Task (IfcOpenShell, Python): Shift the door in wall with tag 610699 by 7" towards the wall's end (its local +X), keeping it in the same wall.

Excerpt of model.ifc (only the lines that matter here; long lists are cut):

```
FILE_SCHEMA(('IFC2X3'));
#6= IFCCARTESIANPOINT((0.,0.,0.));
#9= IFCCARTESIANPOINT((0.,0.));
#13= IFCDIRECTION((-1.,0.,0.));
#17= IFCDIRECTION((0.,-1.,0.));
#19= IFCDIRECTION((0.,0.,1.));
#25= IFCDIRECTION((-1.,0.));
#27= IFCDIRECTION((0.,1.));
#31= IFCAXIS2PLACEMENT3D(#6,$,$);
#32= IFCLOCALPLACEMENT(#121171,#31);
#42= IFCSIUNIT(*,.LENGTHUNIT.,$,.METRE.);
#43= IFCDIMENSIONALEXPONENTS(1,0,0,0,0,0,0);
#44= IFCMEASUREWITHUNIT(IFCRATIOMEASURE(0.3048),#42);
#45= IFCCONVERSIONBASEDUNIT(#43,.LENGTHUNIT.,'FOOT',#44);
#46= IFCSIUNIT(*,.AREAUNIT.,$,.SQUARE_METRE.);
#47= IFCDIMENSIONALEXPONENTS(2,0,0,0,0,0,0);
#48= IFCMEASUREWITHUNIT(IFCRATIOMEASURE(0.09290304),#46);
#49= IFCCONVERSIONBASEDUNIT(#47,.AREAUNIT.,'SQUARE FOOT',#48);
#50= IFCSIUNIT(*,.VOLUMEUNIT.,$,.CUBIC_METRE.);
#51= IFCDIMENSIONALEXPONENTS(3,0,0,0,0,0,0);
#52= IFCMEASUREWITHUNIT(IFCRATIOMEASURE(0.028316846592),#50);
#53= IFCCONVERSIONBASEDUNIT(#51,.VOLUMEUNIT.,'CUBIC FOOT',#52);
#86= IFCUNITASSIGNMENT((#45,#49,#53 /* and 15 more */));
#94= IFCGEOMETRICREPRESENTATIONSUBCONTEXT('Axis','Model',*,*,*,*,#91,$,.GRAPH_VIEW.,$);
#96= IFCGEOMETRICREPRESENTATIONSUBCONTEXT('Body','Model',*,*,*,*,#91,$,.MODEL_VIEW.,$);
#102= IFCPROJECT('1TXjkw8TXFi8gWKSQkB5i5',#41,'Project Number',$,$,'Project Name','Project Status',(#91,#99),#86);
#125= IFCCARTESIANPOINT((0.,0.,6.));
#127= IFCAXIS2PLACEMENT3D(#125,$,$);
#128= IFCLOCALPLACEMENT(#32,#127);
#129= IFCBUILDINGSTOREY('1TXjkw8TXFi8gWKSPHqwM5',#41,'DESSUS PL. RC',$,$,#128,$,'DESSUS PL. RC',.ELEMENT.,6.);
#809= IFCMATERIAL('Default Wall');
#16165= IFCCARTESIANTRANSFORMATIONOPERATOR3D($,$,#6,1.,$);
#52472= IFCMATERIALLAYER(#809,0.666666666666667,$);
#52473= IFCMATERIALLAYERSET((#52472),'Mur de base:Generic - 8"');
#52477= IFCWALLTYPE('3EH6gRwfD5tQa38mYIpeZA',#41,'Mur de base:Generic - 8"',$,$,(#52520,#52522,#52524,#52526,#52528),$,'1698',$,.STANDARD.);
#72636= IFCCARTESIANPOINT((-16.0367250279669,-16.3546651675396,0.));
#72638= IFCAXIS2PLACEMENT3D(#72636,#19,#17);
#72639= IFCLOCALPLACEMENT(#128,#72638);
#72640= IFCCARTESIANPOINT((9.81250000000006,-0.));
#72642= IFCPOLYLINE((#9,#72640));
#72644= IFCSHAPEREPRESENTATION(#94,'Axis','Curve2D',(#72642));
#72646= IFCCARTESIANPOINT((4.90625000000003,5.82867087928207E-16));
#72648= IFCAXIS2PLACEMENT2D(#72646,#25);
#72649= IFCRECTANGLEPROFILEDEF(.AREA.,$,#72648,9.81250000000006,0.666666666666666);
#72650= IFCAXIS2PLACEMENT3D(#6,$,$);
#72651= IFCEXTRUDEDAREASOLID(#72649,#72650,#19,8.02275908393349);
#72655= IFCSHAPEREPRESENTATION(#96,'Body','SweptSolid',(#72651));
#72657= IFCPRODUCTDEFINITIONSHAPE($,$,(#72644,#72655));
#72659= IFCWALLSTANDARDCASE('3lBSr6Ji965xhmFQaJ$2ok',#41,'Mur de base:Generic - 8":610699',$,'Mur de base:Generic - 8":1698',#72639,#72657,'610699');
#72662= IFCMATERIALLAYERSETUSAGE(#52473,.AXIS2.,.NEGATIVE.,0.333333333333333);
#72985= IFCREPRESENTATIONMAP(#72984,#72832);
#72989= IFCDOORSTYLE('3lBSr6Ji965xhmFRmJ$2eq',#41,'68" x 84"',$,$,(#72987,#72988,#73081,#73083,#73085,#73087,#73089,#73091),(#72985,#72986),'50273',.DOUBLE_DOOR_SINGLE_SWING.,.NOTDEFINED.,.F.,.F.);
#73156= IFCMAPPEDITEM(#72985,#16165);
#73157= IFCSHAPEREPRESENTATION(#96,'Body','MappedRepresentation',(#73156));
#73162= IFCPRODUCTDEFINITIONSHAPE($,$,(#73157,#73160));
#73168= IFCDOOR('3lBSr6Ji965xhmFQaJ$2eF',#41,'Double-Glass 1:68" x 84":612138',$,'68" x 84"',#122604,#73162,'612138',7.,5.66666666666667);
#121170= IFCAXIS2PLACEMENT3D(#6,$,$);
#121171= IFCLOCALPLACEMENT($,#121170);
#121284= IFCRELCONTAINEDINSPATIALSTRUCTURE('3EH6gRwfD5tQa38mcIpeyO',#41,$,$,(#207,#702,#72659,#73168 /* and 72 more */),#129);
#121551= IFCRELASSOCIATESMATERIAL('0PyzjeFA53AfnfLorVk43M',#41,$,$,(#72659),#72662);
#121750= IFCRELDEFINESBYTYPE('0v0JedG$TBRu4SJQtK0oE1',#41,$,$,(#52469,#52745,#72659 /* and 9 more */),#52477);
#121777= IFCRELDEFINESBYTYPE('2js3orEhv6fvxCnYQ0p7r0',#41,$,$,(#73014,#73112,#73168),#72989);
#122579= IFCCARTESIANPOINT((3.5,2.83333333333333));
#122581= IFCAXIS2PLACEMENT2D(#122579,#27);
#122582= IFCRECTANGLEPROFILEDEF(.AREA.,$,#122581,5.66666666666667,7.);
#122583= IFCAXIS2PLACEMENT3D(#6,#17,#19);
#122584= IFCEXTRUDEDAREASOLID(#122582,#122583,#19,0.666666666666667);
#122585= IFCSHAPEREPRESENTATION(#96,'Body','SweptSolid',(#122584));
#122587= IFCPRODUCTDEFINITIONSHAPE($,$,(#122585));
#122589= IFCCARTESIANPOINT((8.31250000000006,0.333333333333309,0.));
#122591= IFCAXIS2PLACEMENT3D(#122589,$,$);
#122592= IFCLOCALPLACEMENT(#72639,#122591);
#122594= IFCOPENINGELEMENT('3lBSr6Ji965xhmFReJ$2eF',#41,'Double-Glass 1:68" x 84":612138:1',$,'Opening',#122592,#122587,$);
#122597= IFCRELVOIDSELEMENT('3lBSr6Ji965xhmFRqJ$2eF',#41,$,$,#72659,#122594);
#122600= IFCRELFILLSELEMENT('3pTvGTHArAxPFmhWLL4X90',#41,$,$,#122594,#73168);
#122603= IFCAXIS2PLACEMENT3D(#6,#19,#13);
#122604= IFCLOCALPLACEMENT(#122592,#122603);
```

```python
import ifcopenshell
import ifcopenshell.api.geometry
import ifcopenshell.util.placement
import ifcopenshell.util.unit

model = ifcopenshell.open("model.ifc")
unit_scale = ifcopenshell.util.unit.calculate_unit_scale(model)

door = model.by_id(73168)
opening = door.FillsVoids[0].RelatingOpeningElement
wall = opening.VoidsElements[0].RelatingBuildingElement

wall_matrix = ifcopenshell.util.placement.get_local_placement(wall.ObjectPlacement)
shift = wall_matrix[:3, 0] * 7 * 0.0254 / unit_scale
before = ifcopenshell.util.placement.get_local_placement(door.ObjectPlacement)[:3, 3].copy()

# The door is placed relative to its opening, so it follows when the opening moves.
matrix = ifcopenshell.util.placement.get_local_placement(opening.ObjectPlacement)
matrix[:3, 3] += shift
ifcopenshell.api.geometry.edit_object_placement(
    model, product=opening, matrix=matrix, is_si=False, should_transform_children=True
)

after = ifcopenshell.util.placement.get_local_placement(door.ObjectPlacement)[:3, 3]
print("door moved by", (after - before).round(3) + 0.0)

model.write("model_v2.ifc")
```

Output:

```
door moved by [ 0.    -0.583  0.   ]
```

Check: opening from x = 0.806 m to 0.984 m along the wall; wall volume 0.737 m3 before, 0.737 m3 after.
